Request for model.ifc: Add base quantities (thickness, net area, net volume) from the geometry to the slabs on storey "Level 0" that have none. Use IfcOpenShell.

First a look at what the model holds.

```python
import ifcopenshell
import ifcopenshell.util.element
import ifcopenshell.util.unit

model = ifcopenshell.open("model.ifc")
print(model.schema)
for unit_type in ("LENGTHUNIT", "AREAUNIT", "VOLUMEUNIT"):
    print(unit_type, ifcopenshell.util.unit.calculate_unit_scale(model, unit_type))
storey = next(s for s in model.by_type("IfcBuildingStorey") if s.Name == "Level 0")
slabs = [e for e in ifcopenshell.util.element.get_decomposition(storey) if e.is_a("IfcSlab")]
for e in sorted(slabs, key=lambda e: e.id()):
    print(e.id(), e.is_a(), e.Name, list(ifcopenshell.util.element.get_psets(e, qtos_only=True)), sep=" | ")
```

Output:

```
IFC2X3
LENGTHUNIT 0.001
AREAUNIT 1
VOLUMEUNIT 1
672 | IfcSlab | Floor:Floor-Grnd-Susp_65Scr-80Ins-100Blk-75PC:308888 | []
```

```python
import ifcopenshell
import ifcopenshell.api.pset
import ifcopenshell.geom
import ifcopenshell.util.element
import ifcopenshell.util.shape
import ifcopenshell.util.unit

model = ifcopenshell.open("model.ifc")
unit_scale = ifcopenshell.util.unit.calculate_unit_scale(model)
area_scale = ifcopenshell.util.unit.calculate_unit_scale(model, "AREAUNIT")
volume_scale = ifcopenshell.util.unit.calculate_unit_scale(model, "VOLUMEUNIT")
settings = ifcopenshell.geom.settings()

storey = next(s for s in model.by_type("IfcBuildingStorey") if s.Name == "Level 0")
slabs = [e for e in ifcopenshell.util.element.get_decomposition(storey) if e.is_a("IfcSlab")]

for e in sorted(slabs, key=lambda e: e.id()):
    if ifcopenshell.util.element.get_psets(e, qtos_only=True, should_inherit=False):
        continue
    # Geometry comes back in metres, in the element's own axes.
    shape = ifcopenshell.geom.create_shape(settings, e)
    values = {
        "Width": ifcopenshell.util.shape.get_z(shape.geometry) / unit_scale,
        "NetArea": ifcopenshell.util.shape.get_footprint_area(shape.geometry) / area_scale,
        "NetVolume": ifcopenshell.util.shape.get_volume(shape.geometry) / volume_scale,
    }
    qto = ifcopenshell.api.pset.add_qto(model, product=e, name="BaseQuantities")
    ifcopenshell.api.pset.edit_qto(model, qto=qto, properties=values)
    print(e.id(), {k: round(v, 3) for k, v in values.items()})

model.write("model-out.ifc")
```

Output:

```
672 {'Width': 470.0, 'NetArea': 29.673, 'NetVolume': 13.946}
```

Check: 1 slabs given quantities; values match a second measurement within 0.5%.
